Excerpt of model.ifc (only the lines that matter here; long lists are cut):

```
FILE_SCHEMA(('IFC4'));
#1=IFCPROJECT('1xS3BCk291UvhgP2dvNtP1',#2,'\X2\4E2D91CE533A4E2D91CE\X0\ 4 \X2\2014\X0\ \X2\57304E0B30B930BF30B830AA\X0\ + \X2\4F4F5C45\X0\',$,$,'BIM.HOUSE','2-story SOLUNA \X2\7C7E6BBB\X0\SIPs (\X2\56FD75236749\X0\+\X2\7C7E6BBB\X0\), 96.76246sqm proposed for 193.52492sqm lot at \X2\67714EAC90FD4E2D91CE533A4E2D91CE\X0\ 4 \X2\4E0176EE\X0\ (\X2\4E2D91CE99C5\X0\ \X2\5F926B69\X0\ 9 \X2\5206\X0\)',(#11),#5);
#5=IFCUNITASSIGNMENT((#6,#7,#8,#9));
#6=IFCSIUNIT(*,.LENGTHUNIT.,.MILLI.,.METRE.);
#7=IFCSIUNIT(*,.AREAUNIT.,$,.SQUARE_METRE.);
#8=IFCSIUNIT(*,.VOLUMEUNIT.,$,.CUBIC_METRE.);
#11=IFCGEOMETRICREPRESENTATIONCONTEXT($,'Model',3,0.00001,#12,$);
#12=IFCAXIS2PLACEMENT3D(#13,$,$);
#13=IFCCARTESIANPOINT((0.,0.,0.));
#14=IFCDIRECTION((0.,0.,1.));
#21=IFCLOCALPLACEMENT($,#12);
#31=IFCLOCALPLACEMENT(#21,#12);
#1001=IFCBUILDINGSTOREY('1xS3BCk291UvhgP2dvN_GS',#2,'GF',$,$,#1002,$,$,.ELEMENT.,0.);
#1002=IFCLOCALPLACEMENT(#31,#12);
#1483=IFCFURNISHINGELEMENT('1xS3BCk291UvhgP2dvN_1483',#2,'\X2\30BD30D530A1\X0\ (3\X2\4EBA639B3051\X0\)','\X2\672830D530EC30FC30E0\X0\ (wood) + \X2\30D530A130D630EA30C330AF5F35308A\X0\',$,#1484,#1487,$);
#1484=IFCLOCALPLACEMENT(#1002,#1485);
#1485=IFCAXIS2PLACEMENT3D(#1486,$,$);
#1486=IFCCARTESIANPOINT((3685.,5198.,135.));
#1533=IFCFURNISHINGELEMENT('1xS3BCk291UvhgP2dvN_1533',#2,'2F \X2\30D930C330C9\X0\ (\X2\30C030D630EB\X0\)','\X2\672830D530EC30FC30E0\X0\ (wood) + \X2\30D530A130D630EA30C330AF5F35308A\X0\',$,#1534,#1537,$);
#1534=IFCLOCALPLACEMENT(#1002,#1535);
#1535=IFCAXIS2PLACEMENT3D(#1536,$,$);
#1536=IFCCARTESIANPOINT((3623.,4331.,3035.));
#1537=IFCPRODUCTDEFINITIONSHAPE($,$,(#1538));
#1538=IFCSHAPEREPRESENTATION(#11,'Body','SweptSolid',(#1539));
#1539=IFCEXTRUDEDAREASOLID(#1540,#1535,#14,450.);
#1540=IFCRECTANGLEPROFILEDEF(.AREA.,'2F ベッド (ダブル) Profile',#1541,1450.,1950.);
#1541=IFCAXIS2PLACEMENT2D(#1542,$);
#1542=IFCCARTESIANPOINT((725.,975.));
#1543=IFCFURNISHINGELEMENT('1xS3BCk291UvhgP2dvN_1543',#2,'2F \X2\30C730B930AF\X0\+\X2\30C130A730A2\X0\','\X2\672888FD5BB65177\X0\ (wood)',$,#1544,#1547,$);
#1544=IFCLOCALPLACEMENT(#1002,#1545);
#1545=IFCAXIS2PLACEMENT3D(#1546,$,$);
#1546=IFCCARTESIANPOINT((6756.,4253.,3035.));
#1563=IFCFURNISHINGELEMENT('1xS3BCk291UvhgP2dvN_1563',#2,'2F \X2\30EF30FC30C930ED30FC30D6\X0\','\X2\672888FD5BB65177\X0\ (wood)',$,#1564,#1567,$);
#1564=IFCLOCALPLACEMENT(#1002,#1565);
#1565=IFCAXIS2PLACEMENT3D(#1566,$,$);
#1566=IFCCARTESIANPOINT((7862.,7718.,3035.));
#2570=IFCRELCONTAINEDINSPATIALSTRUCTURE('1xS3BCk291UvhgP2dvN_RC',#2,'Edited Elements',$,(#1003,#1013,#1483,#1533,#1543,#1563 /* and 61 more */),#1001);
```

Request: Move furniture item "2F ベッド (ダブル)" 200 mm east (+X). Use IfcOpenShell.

```python
import ifcopenshell
import ifcopenshell.api.geometry
import ifcopenshell.util.placement
import ifcopenshell.util.unit

model = ifcopenshell.open("model.ifc")
unit_scale = ifcopenshell.util.unit.calculate_unit_scale(model)

item = model.by_guid("1xS3BCk291UvhgP2dvN_1533")
matrix = ifcopenshell.util.placement.get_local_placement(item.ObjectPlacement)
matrix[0, 3] += 0.2 / unit_scale
ifcopenshell.api.geometry.edit_object_placement(model, product=item, matrix=matrix, is_si=False)

print(ifcopenshell.util.placement.get_local_placement(item.ObjectPlacement).round(3) + 0.0)

model.write("model_updated.ifc")
```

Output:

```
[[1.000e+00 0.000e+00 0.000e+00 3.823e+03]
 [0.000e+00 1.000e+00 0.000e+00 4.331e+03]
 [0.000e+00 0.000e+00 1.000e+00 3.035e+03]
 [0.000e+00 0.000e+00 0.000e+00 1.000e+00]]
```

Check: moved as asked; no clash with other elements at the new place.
